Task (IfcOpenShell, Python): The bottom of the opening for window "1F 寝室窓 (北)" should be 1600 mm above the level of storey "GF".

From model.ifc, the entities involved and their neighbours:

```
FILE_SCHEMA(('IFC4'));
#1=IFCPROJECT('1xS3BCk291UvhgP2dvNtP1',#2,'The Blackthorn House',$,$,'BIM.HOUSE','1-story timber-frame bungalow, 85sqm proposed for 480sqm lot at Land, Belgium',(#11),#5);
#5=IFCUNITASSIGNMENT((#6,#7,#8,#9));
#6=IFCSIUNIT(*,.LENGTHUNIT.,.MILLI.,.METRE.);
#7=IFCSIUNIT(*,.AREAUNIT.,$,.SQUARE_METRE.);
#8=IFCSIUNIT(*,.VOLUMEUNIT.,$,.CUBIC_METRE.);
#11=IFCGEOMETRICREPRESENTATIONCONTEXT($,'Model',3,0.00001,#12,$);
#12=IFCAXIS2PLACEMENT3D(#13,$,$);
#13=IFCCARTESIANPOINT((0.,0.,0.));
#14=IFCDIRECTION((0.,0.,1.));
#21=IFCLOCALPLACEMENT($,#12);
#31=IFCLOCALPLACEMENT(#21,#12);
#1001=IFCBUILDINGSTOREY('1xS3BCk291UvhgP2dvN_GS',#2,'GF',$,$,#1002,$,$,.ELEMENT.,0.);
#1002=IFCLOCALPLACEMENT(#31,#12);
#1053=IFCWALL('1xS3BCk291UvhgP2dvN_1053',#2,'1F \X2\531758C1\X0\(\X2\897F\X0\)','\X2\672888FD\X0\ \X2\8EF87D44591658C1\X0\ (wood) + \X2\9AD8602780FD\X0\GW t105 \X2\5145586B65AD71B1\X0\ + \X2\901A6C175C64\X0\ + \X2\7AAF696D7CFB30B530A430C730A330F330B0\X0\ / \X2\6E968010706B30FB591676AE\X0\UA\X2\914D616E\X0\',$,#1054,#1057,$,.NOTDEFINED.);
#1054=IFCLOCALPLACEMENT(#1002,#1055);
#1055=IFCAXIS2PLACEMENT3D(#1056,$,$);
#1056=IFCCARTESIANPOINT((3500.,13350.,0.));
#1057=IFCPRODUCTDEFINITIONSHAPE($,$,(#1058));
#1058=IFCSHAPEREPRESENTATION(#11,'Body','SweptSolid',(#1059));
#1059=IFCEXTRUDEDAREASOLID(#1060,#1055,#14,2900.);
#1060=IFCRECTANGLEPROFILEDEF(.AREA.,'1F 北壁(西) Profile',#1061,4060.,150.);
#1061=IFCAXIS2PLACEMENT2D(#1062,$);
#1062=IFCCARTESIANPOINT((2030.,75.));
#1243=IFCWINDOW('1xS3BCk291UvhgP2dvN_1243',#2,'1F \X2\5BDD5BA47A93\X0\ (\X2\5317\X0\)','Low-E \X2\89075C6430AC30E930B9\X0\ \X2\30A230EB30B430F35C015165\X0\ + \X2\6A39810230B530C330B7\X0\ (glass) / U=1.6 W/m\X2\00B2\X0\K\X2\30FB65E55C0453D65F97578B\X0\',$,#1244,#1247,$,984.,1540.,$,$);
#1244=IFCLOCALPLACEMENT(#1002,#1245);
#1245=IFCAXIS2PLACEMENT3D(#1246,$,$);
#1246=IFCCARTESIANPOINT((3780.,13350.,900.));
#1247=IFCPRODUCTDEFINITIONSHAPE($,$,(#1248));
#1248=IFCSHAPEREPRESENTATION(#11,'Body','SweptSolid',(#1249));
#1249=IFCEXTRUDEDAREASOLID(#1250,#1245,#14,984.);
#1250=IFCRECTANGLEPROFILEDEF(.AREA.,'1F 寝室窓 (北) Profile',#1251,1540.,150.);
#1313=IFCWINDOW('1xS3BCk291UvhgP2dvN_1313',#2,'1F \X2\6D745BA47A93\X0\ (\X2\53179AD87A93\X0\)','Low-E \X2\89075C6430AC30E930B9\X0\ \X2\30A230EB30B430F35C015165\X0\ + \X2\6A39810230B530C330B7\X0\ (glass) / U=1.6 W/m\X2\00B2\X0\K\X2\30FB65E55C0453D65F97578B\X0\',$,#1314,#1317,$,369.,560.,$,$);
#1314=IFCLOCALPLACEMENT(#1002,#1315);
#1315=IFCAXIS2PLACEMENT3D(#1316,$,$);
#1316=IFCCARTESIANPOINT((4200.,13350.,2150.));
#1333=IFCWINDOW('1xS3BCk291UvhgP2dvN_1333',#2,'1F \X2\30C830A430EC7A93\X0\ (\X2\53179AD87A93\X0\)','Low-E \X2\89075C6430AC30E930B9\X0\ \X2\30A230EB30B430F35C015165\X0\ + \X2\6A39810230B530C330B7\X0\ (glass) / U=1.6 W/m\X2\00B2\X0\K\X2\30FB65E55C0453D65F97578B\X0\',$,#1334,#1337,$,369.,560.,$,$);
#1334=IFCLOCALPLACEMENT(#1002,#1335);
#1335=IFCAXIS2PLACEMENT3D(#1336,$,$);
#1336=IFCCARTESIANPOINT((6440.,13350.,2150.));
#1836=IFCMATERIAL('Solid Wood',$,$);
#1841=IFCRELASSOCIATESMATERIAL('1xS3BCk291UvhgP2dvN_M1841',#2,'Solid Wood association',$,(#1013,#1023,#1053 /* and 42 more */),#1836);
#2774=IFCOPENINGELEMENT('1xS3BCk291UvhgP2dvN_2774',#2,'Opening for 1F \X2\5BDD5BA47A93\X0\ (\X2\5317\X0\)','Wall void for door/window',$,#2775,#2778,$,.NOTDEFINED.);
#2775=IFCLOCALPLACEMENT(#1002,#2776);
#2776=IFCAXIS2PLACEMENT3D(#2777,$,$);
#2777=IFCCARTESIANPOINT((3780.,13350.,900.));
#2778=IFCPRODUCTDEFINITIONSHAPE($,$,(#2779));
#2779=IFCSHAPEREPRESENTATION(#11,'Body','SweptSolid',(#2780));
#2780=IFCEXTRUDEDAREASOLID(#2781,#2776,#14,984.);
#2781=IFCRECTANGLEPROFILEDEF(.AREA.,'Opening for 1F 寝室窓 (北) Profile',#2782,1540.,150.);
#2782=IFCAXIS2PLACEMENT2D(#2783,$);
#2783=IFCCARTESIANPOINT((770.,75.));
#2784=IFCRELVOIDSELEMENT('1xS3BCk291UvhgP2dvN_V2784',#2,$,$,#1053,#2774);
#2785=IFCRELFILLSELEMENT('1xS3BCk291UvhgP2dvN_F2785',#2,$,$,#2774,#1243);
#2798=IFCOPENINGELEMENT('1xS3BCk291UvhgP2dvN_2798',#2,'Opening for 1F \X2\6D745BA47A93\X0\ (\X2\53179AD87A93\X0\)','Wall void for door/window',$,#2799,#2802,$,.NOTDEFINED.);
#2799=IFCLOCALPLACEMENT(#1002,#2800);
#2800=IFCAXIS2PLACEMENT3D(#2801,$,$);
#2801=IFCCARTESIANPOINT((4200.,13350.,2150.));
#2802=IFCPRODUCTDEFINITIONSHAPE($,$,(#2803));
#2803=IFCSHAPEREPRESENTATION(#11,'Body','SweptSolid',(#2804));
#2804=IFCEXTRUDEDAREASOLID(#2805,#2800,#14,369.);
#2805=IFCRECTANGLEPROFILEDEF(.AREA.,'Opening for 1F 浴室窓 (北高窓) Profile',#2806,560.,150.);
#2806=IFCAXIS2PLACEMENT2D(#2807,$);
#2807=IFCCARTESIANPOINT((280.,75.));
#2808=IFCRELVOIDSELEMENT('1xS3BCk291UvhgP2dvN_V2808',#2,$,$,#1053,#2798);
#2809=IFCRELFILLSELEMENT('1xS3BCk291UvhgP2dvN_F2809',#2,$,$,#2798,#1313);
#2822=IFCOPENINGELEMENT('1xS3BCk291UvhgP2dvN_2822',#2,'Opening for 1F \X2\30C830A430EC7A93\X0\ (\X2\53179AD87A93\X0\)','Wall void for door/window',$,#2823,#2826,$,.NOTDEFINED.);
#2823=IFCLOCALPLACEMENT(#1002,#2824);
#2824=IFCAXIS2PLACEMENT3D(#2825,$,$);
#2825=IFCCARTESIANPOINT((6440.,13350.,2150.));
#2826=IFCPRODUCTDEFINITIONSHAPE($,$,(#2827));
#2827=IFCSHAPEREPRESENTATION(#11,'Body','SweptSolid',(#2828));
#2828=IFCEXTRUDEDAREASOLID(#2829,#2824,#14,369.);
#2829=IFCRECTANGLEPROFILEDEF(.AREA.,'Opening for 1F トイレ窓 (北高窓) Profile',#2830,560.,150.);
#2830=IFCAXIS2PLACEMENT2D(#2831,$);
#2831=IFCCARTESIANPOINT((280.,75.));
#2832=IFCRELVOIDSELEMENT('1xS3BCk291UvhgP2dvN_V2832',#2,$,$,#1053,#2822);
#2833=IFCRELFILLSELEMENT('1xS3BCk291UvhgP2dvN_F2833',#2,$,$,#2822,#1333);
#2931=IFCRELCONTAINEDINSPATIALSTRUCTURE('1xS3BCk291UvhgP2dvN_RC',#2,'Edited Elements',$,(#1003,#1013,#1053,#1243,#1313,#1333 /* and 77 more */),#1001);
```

```python
import numpy as np
import ifcopenshell
import ifcopenshell.api.geometry
import ifcopenshell.geom
import ifcopenshell.util.element
import ifcopenshell.util.placement
import ifcopenshell.util.shape
import ifcopenshell.util.unit

model = ifcopenshell.open("model.ifc")
unit_scale = ifcopenshell.util.unit.calculate_unit_scale(model)

window = model.by_id(1243)
opening = window.FillsVoids[0].RelatingOpeningElement
storey = ifcopenshell.util.element.get_container(window, ifc_class="IfcBuildingStorey")
level = ifcopenshell.util.placement.get_local_placement(storey.ObjectPlacement)[2, 3]

# The opening's origin need not be at the sill, so measure its lowest point.
shape = ifcopenshell.geom.create_shape(ifcopenshell.geom.settings(), opening)
bottom = ifcopenshell.util.shape.get_shape_bottom_elevation(shape, shape.geometry) / unit_scale
dz = level + 1.6 / unit_scale - bottom

shift = np.array([0.0, 0.0, dz])
# The window is not placed relative to its opening, so move both.
for product in (opening, window):
    matrix = ifcopenshell.util.placement.get_local_placement(product.ObjectPlacement)
    matrix[:3, 3] += shift
    ifcopenshell.api.geometry.edit_object_placement(model, product=product, matrix=matrix, is_si=False)

print(f"moved by {dz * unit_scale:+.3f} m")

model.write("model_rev.ifc")
```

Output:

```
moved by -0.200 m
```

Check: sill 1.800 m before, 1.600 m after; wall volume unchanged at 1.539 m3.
